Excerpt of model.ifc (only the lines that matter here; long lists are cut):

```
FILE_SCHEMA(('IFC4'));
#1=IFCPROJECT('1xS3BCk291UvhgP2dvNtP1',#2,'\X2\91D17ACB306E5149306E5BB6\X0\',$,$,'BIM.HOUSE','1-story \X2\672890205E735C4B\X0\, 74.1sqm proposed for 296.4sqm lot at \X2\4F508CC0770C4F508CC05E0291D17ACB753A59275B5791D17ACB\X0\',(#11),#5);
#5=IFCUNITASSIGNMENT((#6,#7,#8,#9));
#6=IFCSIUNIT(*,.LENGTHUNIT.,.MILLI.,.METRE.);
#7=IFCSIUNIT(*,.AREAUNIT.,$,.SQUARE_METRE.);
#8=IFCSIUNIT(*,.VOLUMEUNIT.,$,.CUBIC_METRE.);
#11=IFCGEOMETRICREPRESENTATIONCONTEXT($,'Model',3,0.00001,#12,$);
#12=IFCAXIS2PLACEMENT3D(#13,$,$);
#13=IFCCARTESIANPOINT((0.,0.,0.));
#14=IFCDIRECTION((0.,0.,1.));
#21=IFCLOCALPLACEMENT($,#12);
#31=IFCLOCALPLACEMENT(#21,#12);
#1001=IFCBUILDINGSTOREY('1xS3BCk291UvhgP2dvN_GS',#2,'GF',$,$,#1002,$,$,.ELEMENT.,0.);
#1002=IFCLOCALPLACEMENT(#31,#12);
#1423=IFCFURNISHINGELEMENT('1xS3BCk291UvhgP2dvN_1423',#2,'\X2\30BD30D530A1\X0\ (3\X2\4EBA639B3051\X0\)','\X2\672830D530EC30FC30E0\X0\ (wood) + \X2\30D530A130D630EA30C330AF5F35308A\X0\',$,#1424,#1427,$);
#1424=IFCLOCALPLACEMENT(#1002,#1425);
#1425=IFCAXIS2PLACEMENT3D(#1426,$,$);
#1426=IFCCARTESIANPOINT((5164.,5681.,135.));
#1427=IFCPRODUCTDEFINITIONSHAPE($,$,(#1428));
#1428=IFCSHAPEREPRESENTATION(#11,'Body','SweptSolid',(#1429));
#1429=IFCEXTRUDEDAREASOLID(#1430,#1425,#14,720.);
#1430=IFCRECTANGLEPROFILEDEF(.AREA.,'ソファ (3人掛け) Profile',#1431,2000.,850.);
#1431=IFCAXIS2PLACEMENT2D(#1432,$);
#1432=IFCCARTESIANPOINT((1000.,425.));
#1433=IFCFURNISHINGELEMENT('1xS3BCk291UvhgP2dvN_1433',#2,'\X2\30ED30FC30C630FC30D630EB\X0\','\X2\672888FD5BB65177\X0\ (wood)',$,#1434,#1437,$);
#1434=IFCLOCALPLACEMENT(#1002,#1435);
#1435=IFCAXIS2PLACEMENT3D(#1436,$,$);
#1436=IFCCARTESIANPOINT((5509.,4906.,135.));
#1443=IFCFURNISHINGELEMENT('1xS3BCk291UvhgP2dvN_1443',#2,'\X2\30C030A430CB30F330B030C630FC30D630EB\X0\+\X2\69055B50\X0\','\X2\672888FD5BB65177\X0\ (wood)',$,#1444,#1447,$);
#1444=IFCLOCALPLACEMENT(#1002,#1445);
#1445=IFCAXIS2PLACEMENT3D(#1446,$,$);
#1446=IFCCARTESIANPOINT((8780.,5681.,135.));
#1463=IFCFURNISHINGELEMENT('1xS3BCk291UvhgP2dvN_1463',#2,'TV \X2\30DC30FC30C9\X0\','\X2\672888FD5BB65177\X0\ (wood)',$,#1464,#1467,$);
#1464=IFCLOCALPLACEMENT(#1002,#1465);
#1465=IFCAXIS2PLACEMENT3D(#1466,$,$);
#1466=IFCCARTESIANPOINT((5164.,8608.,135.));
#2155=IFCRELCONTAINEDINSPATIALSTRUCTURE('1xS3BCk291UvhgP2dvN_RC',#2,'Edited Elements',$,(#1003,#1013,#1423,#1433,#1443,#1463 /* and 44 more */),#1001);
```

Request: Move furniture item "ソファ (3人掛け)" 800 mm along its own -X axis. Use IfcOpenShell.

```python
import ifcopenshell
import ifcopenshell.api.geometry
import ifcopenshell.util.placement

model = ifcopenshell.open("model.ifc")

item = model.by_guid("1xS3BCk291UvhgP2dvN_1423")
matrix = ifcopenshell.util.placement.get_local_placement(item.ObjectPlacement)
matrix[:3, 3] -= matrix[:3, 0] * 800.0
ifcopenshell.api.geometry.edit_object_placement(model, product=item, matrix=matrix, is_si=False)

print(ifcopenshell.util.placement.get_local_placement(item.ObjectPlacement).round(3) + 0.0)

model.write("model_v2.ifc")
```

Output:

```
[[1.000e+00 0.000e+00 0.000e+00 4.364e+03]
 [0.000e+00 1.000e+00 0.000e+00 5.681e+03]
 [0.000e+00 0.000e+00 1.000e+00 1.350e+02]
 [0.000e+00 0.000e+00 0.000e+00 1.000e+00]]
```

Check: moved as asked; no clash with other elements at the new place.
